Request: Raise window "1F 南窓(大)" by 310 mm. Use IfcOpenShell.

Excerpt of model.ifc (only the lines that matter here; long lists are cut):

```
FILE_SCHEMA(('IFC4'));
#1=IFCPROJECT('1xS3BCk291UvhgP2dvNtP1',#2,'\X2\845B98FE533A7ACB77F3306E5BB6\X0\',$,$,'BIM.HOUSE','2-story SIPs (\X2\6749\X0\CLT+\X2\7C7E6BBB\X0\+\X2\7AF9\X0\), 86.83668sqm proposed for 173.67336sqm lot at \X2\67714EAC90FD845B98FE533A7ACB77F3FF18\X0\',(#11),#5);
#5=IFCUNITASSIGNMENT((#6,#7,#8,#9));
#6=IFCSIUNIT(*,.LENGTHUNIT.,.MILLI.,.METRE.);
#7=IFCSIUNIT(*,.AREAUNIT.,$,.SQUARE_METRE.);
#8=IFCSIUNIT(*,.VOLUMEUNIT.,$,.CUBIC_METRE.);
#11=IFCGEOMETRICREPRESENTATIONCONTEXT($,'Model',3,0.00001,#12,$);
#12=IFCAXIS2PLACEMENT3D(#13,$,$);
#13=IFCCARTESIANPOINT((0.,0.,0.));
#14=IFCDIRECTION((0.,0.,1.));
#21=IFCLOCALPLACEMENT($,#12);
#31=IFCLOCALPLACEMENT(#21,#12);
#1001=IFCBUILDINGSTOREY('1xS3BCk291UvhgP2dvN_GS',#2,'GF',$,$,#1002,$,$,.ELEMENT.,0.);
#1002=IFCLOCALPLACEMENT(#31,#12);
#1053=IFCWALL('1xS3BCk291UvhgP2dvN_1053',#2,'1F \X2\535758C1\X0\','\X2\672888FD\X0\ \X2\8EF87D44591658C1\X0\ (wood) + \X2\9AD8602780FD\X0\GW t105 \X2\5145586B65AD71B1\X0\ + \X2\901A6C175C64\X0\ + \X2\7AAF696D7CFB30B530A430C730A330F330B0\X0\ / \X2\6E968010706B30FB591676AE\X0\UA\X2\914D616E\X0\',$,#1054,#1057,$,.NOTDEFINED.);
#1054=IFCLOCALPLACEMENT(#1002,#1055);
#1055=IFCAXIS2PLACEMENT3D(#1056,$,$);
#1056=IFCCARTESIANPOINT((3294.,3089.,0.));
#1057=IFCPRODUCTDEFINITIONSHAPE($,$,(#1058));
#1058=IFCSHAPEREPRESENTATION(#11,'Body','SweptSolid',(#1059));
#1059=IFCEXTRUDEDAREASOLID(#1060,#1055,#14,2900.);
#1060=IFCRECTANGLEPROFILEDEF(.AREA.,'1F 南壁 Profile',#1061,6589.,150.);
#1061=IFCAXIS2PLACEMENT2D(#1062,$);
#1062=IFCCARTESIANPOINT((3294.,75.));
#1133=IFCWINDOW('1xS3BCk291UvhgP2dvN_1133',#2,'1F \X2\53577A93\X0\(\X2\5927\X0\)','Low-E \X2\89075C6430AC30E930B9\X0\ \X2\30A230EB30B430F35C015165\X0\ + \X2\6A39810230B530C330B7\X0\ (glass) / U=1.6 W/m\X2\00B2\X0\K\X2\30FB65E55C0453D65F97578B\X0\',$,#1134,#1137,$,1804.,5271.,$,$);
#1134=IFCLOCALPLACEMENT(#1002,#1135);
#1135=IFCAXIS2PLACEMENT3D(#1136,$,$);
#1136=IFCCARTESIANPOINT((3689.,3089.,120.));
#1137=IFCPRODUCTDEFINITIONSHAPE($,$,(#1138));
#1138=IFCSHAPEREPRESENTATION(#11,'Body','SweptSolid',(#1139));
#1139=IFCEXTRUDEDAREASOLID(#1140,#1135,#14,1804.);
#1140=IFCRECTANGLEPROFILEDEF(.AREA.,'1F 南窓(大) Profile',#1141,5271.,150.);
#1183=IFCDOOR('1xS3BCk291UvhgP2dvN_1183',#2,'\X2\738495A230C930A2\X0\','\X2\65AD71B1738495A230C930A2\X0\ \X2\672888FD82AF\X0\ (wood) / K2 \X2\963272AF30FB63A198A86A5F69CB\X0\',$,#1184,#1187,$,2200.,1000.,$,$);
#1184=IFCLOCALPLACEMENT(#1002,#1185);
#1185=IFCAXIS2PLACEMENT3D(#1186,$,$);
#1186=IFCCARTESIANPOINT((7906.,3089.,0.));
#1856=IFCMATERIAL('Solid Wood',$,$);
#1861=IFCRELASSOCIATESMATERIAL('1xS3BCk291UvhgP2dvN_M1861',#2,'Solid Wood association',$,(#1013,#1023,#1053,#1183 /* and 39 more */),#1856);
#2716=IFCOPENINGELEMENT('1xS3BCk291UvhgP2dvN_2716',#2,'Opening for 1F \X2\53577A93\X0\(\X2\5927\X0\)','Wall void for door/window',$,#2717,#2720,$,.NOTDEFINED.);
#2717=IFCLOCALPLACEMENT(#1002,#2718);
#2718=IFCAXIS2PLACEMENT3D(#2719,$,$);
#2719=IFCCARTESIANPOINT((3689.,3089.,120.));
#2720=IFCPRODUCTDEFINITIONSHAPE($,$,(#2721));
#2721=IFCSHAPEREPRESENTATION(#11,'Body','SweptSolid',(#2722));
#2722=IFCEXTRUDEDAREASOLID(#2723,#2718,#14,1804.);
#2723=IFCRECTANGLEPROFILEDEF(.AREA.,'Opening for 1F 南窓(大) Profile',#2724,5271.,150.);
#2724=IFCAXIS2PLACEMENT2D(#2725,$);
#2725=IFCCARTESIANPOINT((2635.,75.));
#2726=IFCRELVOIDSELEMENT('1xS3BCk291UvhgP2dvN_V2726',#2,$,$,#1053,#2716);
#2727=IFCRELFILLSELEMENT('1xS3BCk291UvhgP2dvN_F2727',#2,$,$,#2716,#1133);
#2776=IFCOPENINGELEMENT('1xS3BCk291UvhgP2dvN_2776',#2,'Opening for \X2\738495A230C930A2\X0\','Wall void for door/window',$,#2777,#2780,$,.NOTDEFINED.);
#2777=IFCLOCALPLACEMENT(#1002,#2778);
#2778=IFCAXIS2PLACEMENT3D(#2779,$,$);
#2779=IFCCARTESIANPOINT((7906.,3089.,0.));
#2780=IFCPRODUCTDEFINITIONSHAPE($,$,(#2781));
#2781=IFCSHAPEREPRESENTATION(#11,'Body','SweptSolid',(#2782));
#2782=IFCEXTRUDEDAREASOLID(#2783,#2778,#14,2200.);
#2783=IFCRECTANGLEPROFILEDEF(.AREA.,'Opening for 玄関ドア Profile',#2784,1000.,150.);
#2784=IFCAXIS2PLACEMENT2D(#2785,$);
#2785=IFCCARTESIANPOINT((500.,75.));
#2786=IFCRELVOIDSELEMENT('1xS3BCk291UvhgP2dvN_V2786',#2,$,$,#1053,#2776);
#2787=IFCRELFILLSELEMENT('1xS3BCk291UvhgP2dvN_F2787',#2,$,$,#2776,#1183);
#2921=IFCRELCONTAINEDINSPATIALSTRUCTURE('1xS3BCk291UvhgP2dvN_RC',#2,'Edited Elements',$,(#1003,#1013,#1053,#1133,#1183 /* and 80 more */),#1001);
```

```python
import numpy as np
import ifcopenshell
import ifcopenshell.api.geometry
import ifcopenshell.util.placement
import ifcopenshell.util.unit

model = ifcopenshell.open("model.ifc")
unit_scale = ifcopenshell.util.unit.calculate_unit_scale(model)

window = model.by_guid("1xS3BCk291UvhgP2dvN_1133")
opening = window.FillsVoids[0].RelatingOpeningElement
dz = 310.0

shift = np.array([0.0, 0.0, dz])
# The window is not placed relative to its opening, so move both.
for product in (opening, window):
    matrix = ifcopenshell.util.placement.get_local_placement(product.ObjectPlacement)
    matrix[:3, 3] += shift
    ifcopenshell.api.geometry.edit_object_placement(model, product=product, matrix=matrix, is_si=False)

print(f"moved by {dz * unit_scale:+.3f} m")

model.write("model_updated.ifc")
```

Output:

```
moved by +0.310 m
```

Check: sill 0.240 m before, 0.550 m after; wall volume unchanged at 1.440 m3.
